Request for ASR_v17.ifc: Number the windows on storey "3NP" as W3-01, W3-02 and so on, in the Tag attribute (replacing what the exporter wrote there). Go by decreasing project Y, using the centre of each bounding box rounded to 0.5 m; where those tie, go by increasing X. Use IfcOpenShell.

First a look at what the model holds.

```python
import ifcopenshell
import ifcopenshell.util.element
import ifcopenshell.util.placement

model = ifcopenshell.open("ASR_v17.ifc")
print(model.schema)
storey = next(s for s in model.by_type("IfcBuildingStorey") if s.Name == "3NP")
windows = [e for e in ifcopenshell.util.element.get_decomposition(storey) if e.is_a("IfcWindow")]
for e in sorted(windows, key=lambda e: e.id()):
    origin = ifcopenshell.util.placement.get_local_placement(e.ObjectPlacement)[:3, 3]
    print(e.id(), e.Tag, e.Name, origin.round(2) + 0.0, sep=" | ")
```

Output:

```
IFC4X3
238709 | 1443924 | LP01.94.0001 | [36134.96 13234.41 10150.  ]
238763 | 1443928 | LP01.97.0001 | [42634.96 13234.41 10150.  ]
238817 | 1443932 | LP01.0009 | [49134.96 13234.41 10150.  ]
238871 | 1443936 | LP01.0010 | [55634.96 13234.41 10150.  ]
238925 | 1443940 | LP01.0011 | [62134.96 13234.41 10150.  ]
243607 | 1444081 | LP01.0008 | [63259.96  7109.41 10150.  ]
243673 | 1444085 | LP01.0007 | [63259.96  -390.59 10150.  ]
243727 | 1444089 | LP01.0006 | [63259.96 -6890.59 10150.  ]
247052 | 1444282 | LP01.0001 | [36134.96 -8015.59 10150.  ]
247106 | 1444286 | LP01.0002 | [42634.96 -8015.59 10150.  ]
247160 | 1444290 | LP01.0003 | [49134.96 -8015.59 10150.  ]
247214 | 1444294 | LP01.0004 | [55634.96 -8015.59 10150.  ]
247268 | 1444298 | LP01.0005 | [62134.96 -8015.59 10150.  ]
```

```python
import ifcopenshell
import ifcopenshell.geom
import ifcopenshell.util.element
import ifcopenshell.util.shape

model = ifcopenshell.open("ASR_v17.ifc")
settings = ifcopenshell.geom.settings()
settings.set("use-world-coords", True)


def centre(element):
    shape = ifcopenshell.geom.create_shape(settings, element)
    return ifcopenshell.util.shape.get_bbox_centroid(shape.geometry)


storey = next(s for s in model.by_type("IfcBuildingStorey") if s.Name == "3NP")
windows = [e for e in ifcopenshell.util.element.get_decomposition(storey) if e.is_a("IfcWindow")]

# Insertion points can sit at a corner or the storey origin, so sort by the geometry (in metres).
centres = {e: centre(e) for e in windows}
windows.sort(key=lambda e: (-round(centres[e][1] / 0.5), centres[e][0]))

for i, e in enumerate(windows, start=1):
    number = f"W3-{i:02d}"
    e.Tag = number
    print(e.id(), number)

model.write("ASR_v17_v2.ifc")
```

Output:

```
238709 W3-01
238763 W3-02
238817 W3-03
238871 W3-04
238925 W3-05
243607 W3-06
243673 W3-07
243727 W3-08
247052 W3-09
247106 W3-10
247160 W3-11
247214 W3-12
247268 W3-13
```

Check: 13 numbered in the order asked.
